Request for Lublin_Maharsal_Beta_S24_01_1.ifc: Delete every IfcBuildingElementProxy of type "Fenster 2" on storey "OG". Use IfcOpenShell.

First a look at what the model holds.

```python
import ifcopenshell
import ifcopenshell.util.element

model = ifcopenshell.open("Lublin_Maharsal_Beta_S24_01_1.ifc")
print(model.schema)
storey = next(s for s in model.by_type("IfcBuildingStorey") if s.Name == "OG")
proxies = [e for e in ifcopenshell.util.element.get_decomposition(storey) if e.is_a("IfcBuildingElementProxy")]
seen = {}
for e in proxies:
    element_type = ifcopenshell.util.element.get_type(e)
    name = element_type.Name if element_type not in (None, e) else None
    seen[name] = seen.get(name, 0) + 1
for name, count in sorted(seen.items(), key=str):
    print(count, "x", name)
```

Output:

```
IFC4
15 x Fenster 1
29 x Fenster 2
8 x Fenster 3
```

```python
import ifcopenshell
import ifcopenshell.api.root
import ifcopenshell.util.element

model = ifcopenshell.open("Lublin_Maharsal_Beta_S24_01_1.ifc")

storey = next(s for s in model.by_type("IfcBuildingStorey") if s.Name == "OG")
proxies = [e for e in ifcopenshell.util.element.get_decomposition(storey) if e.is_a("IfcBuildingElementProxy")]
targets = [e for e in proxies if (t := ifcopenshell.util.element.get_type(e)) not in (None, e) and t.Name == "Fenster 2"]

for e in targets:
    ifcopenshell.api.root.remove_product(model, product=e)
print(len(targets), "removed")

model.write("Lublin_Maharsal_Beta_S24_01_1-out.ifc")
```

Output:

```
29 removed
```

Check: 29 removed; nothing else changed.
